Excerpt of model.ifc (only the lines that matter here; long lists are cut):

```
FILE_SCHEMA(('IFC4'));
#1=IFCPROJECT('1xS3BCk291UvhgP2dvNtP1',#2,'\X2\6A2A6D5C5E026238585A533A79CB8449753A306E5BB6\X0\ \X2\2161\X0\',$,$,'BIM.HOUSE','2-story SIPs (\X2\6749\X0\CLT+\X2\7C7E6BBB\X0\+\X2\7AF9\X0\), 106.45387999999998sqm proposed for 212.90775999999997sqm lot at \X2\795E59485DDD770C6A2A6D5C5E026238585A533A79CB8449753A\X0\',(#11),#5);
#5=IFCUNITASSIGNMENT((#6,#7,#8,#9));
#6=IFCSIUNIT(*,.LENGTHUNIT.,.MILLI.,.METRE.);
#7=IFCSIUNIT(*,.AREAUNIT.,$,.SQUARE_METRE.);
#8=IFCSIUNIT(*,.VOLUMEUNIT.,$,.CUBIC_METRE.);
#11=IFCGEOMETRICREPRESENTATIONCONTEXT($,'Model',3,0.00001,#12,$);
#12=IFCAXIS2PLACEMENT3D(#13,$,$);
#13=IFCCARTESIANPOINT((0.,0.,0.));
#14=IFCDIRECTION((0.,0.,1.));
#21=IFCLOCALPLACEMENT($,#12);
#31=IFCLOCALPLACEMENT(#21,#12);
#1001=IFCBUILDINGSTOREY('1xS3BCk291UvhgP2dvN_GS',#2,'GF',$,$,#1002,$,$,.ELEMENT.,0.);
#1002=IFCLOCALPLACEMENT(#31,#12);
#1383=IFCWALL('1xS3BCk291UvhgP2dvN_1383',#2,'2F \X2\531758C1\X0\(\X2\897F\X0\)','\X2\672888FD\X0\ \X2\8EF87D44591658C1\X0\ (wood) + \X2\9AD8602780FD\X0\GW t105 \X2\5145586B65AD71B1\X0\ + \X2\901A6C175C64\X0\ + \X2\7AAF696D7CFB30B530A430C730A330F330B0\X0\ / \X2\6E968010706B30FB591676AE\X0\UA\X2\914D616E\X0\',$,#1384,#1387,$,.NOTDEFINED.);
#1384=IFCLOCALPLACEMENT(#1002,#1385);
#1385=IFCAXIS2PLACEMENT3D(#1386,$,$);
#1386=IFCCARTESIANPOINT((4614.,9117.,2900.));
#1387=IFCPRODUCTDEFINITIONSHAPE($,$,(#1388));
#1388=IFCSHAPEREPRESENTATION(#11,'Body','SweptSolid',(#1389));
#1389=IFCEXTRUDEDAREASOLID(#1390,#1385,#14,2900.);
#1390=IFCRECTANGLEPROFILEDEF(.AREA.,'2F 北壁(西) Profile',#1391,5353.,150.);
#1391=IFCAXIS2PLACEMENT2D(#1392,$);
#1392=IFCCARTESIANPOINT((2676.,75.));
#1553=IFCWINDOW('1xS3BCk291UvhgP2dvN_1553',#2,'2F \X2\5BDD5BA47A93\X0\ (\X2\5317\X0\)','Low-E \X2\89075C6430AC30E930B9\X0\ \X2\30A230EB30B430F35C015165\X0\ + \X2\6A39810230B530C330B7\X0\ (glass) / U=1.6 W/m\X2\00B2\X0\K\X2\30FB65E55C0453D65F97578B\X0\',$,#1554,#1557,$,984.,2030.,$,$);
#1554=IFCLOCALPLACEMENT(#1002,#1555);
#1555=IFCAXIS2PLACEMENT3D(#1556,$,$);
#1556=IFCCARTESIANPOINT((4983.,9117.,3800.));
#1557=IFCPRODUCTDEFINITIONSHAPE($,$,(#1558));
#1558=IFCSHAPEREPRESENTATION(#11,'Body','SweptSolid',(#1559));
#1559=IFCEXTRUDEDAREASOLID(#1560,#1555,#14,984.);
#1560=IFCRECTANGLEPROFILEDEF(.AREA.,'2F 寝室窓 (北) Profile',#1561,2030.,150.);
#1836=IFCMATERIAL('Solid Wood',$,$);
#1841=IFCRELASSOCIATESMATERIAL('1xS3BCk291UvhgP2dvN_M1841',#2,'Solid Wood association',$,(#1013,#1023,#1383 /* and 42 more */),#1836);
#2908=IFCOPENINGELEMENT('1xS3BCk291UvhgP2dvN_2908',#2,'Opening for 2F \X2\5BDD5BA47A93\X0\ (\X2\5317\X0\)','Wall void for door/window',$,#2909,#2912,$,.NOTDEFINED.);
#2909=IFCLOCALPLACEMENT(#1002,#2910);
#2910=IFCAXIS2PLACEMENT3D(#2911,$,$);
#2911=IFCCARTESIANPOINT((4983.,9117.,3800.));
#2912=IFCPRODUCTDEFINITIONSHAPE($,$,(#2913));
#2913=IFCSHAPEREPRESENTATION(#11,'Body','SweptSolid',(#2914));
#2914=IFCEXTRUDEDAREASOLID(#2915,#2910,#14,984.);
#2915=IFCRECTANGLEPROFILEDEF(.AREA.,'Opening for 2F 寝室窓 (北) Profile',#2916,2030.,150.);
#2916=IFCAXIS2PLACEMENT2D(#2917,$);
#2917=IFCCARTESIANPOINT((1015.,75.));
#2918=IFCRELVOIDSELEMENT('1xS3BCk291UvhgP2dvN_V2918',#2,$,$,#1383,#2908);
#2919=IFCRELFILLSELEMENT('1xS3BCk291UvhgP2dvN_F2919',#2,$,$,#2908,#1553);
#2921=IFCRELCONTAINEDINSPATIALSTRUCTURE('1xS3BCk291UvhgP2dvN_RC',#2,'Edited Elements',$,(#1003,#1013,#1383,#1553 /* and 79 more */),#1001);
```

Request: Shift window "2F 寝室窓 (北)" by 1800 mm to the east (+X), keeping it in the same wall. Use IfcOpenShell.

```python
import ifcopenshell
import ifcopenshell.api.geometry
import ifcopenshell.util.placement
import ifcopenshell.util.unit

model = ifcopenshell.open("model.ifc")
unit_scale = ifcopenshell.util.unit.calculate_unit_scale(model)

window = model.by_id(1553)
opening = window.FillsVoids[0].RelatingOpeningElement
wall = opening.VoidsElements[0].RelatingBuildingElement

wall_matrix = ifcopenshell.util.placement.get_local_placement(wall.ObjectPlacement)
shift = wall_matrix[:3, 0] * 1.8 / unit_scale
before = ifcopenshell.util.placement.get_local_placement(window.ObjectPlacement)[:3, 3].copy()

# The window is not placed relative to its opening, so move both.
for product in (opening, window):
    matrix = ifcopenshell.util.placement.get_local_placement(product.ObjectPlacement)
    matrix[:3, 3] += shift
    ifcopenshell.api.geometry.edit_object_placement(model, product=product, matrix=matrix, is_si=False)

after = ifcopenshell.util.placement.get_local_placement(window.ObjectPlacement)[:3, 3]
print("window moved by", (after - before).round(3) + 0.0)

model.write("model_updated.ifc")
```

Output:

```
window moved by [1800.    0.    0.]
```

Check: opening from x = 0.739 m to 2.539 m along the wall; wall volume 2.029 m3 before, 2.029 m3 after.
